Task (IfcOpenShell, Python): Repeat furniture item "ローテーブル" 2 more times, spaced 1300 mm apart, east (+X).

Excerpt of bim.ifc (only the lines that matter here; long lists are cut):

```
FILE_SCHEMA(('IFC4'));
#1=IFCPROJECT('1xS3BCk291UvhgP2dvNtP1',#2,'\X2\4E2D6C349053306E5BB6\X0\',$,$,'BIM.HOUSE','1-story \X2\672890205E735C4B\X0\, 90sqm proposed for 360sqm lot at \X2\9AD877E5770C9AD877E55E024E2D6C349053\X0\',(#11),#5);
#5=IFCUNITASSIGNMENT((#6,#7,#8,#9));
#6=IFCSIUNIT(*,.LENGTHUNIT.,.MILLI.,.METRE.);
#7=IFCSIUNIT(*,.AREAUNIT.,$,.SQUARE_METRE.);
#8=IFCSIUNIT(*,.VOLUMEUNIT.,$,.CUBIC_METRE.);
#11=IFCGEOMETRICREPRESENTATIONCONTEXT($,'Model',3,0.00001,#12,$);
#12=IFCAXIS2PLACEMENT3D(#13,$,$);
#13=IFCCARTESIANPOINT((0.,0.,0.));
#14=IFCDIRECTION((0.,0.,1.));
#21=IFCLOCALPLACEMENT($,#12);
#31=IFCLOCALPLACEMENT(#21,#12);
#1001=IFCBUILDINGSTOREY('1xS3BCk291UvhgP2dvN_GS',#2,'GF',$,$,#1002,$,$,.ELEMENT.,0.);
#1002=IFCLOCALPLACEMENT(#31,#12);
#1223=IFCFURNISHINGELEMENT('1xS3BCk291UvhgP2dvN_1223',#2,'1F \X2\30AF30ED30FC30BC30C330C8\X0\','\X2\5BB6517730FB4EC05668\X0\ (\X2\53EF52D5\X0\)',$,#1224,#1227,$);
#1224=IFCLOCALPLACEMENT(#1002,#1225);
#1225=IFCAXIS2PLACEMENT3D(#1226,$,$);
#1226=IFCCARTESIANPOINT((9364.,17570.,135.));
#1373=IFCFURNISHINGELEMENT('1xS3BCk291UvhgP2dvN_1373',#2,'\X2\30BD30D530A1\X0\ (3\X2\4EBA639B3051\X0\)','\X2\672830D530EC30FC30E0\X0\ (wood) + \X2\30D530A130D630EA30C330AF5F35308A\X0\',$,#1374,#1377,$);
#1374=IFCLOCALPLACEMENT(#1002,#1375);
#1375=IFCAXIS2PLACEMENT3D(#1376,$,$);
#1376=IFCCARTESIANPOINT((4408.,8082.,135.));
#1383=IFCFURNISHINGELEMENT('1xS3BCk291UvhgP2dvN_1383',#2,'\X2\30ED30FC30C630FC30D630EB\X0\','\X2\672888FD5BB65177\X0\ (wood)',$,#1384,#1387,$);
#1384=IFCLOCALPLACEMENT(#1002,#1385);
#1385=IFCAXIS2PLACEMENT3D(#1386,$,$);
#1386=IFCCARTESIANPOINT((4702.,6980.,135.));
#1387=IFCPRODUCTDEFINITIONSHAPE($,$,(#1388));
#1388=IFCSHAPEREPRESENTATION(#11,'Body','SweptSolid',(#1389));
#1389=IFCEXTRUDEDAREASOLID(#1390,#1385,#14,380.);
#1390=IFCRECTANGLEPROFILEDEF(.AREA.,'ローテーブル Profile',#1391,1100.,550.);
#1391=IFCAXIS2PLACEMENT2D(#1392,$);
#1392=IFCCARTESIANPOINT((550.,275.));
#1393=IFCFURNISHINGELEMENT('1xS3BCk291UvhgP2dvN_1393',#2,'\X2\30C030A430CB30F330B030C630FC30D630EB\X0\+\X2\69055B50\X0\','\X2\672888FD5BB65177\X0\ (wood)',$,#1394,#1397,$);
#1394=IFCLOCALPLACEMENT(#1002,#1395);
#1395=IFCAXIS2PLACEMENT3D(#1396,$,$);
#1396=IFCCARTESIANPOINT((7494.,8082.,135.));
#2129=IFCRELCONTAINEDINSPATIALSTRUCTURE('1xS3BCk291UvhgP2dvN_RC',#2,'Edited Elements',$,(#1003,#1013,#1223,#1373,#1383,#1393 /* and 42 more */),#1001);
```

```python
import numpy as np
import ifcopenshell
import ifcopenshell.api.geometry
import ifcopenshell.api.root
import ifcopenshell.util.element
import ifcopenshell.util.placement

model = ifcopenshell.open("bim.ifc")


def reuse_history(source, copy):
    """copy_class also copies each property set's owner history, people and application; keep the originals."""
    for rel in copy.IsDefinedBy:
        if rel.is_a("IfcRelDefinesByProperties") and (history := rel.RelatingPropertyDefinition.OwnerHistory):
            rel.RelatingPropertyDefinition.OwnerHistory = source.OwnerHistory
            ifcopenshell.util.element.remove_deep2(model, history)


source = model.by_guid("1xS3BCk291UvhgP2dvN_1383")
base = ifcopenshell.util.placement.get_local_placement(source.ObjectPlacement)
step = np.array([1.0, 0.0, 0.0]) * 1300.0

for i in range(1, 3):
    copy = ifcopenshell.api.root.copy_class(model, product=source)
    copy.Representation = ifcopenshell.util.element.copy_deep(
        model, source.Representation, exclude=["IfcGeometricRepresentationContext", "IfcRepresentationMap"]
    )
    reuse_history(source, copy)
    matrix = base.copy()
    matrix[:3, 3] += i * step
    print("added at", matrix[:3, 3].round(3) + 0.0)
    ifcopenshell.api.geometry.edit_object_placement(model, product=copy, matrix=matrix, is_si=False)

model.write("bim_v2.ifc")
```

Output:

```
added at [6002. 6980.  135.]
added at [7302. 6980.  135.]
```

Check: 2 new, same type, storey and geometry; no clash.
